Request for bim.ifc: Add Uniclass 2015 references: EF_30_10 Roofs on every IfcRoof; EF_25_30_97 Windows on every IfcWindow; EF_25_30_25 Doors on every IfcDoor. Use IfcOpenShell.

First a look at what the model holds.

```python
import ifcopenshell

model = ifcopenshell.open("bim.ifc")
print(model.schema)
print("classifications:", [c.Name for c in model.by_type("IfcClassification")])
for ifc_class in ("IfcDoor", "IfcRoof", "IfcStair", "IfcWall", "IfcWindow"):
    print(ifc_class, len(model.by_type(ifc_class)))
```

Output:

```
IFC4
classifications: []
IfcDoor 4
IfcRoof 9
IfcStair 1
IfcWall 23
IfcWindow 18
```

```python
import ifcopenshell
import ifcopenshell.api.classification

model = ifcopenshell.open("bim.ifc")

system = ifcopenshell.api.classification.add_classification(model, classification="Uniclass 2015")

codes = {
    "IfcRoof": ("EF_30_10", "Roofs"),
    "IfcWindow": ("EF_25_30_97", "Windows"),
    "IfcDoor": ("EF_25_30_25", "Doors"),
}
for ifc_class, (code, name) in codes.items():
    products = model.by_type(ifc_class)
    ifcopenshell.api.classification.add_reference(
        model, products=products, classification=system, identification=code, name=name
    )
    print(code, len(products))

model.write("bim_updated.ifc")
```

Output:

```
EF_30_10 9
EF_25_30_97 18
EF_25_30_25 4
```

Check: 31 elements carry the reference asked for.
